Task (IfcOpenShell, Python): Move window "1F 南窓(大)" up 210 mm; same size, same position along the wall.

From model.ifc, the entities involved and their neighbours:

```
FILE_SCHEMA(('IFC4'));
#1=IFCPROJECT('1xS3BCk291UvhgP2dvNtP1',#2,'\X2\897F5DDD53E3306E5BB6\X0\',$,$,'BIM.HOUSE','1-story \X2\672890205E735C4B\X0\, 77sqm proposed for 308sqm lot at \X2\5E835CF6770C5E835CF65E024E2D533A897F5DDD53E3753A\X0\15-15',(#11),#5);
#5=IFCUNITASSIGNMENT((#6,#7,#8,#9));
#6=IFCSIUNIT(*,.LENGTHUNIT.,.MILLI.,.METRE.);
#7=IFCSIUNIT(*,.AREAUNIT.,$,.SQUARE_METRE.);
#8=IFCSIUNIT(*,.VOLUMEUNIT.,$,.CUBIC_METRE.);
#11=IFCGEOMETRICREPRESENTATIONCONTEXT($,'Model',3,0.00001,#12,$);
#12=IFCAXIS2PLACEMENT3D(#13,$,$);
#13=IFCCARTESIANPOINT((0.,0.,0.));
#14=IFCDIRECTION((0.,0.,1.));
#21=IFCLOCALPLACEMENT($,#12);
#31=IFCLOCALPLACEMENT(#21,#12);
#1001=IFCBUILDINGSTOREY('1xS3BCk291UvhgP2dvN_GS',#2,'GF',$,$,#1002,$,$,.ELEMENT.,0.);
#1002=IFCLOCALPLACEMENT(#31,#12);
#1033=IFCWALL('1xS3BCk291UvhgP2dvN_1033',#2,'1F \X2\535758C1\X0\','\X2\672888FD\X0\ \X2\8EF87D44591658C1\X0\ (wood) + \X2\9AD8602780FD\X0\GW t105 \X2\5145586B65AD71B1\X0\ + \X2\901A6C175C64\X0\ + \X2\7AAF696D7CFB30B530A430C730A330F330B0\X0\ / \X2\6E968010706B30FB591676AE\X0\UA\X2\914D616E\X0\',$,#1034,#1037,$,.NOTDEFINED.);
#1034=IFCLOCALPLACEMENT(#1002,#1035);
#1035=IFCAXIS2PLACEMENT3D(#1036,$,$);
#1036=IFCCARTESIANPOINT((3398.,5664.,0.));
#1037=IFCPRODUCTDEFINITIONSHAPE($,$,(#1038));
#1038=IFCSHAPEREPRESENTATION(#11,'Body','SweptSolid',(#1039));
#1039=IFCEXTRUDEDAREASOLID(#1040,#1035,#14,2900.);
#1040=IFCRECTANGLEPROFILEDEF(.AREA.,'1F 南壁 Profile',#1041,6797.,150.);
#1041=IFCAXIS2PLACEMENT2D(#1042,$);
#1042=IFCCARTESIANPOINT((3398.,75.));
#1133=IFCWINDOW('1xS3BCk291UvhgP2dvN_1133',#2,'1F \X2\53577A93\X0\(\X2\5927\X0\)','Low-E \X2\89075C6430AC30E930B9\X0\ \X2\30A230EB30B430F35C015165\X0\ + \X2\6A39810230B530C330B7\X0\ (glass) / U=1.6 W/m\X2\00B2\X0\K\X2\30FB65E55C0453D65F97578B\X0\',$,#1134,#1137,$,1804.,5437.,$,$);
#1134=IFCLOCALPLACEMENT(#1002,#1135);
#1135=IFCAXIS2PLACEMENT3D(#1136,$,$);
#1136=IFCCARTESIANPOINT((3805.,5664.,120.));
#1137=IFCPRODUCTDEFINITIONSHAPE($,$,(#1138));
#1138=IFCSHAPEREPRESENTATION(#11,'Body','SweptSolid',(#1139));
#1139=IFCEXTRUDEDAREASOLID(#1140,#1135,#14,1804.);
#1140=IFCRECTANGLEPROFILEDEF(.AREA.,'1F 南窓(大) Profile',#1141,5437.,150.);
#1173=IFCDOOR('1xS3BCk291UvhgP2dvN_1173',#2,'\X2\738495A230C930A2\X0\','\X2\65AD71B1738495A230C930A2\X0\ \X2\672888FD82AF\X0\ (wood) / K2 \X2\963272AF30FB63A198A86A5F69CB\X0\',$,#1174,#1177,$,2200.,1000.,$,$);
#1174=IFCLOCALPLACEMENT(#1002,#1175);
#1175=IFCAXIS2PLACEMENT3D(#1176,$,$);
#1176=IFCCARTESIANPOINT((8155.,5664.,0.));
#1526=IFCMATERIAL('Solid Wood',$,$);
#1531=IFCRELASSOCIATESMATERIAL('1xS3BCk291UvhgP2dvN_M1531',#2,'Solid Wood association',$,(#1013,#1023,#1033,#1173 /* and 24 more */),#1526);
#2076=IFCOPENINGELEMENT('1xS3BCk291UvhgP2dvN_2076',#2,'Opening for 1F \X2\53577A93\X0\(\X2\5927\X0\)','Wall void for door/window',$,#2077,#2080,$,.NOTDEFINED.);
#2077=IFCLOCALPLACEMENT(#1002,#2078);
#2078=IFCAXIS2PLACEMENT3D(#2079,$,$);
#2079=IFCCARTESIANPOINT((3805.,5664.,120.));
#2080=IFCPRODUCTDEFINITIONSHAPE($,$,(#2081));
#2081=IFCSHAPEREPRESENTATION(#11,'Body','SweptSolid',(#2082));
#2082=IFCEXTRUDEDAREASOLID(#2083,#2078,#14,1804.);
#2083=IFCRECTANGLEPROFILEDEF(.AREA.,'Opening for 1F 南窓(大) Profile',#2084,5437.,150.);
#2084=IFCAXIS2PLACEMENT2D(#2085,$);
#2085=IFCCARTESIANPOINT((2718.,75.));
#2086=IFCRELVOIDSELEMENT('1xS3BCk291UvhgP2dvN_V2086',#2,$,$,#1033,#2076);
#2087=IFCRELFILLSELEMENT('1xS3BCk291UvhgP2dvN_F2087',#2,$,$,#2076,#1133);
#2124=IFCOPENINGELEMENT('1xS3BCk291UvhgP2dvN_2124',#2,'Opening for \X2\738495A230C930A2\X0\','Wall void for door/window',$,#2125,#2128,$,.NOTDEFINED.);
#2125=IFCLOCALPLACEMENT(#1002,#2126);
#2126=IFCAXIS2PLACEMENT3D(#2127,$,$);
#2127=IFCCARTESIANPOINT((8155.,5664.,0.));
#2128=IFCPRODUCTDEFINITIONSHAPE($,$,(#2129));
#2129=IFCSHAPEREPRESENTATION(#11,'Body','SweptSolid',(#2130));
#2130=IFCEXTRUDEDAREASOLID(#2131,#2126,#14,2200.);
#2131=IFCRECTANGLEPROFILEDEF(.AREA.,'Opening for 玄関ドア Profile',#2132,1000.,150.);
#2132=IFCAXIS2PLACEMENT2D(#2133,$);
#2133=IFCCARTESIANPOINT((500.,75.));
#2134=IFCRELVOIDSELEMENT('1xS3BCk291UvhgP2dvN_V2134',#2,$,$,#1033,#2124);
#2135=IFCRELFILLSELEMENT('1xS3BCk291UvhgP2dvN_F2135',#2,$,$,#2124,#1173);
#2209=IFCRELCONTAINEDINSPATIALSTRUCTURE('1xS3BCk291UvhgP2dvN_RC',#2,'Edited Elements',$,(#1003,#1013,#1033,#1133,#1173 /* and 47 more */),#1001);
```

```python
import numpy as np
import ifcopenshell
import ifcopenshell.api.geometry
import ifcopenshell.util.placement
import ifcopenshell.util.unit

model = ifcopenshell.open("model.ifc")
unit_scale = ifcopenshell.util.unit.calculate_unit_scale(model)

window = model.by_guid("1xS3BCk291UvhgP2dvN_1133")
opening = window.FillsVoids[0].RelatingOpeningElement
dz = 210.0

shift = np.array([0.0, 0.0, dz])
# The window is not placed relative to its opening, so move both.
for product in (opening, window):
    matrix = ifcopenshell.util.placement.get_local_placement(product.ObjectPlacement)
    matrix[:3, 3] += shift
    ifcopenshell.api.geometry.edit_object_placement(model, product=product, matrix=matrix, is_si=False)

print(f"moved by {dz * unit_scale:+.3f} m")

model.write("model_v2.ifc")
```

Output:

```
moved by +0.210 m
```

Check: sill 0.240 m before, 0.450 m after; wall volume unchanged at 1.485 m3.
